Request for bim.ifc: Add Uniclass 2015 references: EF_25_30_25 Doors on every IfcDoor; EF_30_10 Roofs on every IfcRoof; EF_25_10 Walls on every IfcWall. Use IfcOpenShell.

First a look at what the model holds.

```python
import ifcopenshell

model = ifcopenshell.open("bim.ifc")
print(model.schema)
print("classifications:", [c.Name for c in model.by_type("IfcClassification")])
for ifc_class in ("IfcDoor", "IfcRoof", "IfcStair", "IfcWall", "IfcWindow"):
    print(ifc_class, len(model.by_type(ifc_class)))
```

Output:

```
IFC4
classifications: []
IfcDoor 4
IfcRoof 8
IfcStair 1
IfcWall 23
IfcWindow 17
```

```python
import ifcopenshell
import ifcopenshell.api.classification

model = ifcopenshell.open("bim.ifc")

system = ifcopenshell.api.classification.add_classification(model, classification="Uniclass 2015")

codes = {
    "IfcDoor": ("EF_25_30_25", "Doors"),
    "IfcRoof": ("EF_30_10", "Roofs"),
    "IfcWall": ("EF_25_10", "Walls"),
}
for ifc_class, (code, name) in codes.items():
    products = model.by_type(ifc_class)
    ifcopenshell.api.classification.add_reference(
        model, products=products, classification=system, identification=code, name=name
    )
    print(code, len(products))

model.write("bim_v2.ifc")
```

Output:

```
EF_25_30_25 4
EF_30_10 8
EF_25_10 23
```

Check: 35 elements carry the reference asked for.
